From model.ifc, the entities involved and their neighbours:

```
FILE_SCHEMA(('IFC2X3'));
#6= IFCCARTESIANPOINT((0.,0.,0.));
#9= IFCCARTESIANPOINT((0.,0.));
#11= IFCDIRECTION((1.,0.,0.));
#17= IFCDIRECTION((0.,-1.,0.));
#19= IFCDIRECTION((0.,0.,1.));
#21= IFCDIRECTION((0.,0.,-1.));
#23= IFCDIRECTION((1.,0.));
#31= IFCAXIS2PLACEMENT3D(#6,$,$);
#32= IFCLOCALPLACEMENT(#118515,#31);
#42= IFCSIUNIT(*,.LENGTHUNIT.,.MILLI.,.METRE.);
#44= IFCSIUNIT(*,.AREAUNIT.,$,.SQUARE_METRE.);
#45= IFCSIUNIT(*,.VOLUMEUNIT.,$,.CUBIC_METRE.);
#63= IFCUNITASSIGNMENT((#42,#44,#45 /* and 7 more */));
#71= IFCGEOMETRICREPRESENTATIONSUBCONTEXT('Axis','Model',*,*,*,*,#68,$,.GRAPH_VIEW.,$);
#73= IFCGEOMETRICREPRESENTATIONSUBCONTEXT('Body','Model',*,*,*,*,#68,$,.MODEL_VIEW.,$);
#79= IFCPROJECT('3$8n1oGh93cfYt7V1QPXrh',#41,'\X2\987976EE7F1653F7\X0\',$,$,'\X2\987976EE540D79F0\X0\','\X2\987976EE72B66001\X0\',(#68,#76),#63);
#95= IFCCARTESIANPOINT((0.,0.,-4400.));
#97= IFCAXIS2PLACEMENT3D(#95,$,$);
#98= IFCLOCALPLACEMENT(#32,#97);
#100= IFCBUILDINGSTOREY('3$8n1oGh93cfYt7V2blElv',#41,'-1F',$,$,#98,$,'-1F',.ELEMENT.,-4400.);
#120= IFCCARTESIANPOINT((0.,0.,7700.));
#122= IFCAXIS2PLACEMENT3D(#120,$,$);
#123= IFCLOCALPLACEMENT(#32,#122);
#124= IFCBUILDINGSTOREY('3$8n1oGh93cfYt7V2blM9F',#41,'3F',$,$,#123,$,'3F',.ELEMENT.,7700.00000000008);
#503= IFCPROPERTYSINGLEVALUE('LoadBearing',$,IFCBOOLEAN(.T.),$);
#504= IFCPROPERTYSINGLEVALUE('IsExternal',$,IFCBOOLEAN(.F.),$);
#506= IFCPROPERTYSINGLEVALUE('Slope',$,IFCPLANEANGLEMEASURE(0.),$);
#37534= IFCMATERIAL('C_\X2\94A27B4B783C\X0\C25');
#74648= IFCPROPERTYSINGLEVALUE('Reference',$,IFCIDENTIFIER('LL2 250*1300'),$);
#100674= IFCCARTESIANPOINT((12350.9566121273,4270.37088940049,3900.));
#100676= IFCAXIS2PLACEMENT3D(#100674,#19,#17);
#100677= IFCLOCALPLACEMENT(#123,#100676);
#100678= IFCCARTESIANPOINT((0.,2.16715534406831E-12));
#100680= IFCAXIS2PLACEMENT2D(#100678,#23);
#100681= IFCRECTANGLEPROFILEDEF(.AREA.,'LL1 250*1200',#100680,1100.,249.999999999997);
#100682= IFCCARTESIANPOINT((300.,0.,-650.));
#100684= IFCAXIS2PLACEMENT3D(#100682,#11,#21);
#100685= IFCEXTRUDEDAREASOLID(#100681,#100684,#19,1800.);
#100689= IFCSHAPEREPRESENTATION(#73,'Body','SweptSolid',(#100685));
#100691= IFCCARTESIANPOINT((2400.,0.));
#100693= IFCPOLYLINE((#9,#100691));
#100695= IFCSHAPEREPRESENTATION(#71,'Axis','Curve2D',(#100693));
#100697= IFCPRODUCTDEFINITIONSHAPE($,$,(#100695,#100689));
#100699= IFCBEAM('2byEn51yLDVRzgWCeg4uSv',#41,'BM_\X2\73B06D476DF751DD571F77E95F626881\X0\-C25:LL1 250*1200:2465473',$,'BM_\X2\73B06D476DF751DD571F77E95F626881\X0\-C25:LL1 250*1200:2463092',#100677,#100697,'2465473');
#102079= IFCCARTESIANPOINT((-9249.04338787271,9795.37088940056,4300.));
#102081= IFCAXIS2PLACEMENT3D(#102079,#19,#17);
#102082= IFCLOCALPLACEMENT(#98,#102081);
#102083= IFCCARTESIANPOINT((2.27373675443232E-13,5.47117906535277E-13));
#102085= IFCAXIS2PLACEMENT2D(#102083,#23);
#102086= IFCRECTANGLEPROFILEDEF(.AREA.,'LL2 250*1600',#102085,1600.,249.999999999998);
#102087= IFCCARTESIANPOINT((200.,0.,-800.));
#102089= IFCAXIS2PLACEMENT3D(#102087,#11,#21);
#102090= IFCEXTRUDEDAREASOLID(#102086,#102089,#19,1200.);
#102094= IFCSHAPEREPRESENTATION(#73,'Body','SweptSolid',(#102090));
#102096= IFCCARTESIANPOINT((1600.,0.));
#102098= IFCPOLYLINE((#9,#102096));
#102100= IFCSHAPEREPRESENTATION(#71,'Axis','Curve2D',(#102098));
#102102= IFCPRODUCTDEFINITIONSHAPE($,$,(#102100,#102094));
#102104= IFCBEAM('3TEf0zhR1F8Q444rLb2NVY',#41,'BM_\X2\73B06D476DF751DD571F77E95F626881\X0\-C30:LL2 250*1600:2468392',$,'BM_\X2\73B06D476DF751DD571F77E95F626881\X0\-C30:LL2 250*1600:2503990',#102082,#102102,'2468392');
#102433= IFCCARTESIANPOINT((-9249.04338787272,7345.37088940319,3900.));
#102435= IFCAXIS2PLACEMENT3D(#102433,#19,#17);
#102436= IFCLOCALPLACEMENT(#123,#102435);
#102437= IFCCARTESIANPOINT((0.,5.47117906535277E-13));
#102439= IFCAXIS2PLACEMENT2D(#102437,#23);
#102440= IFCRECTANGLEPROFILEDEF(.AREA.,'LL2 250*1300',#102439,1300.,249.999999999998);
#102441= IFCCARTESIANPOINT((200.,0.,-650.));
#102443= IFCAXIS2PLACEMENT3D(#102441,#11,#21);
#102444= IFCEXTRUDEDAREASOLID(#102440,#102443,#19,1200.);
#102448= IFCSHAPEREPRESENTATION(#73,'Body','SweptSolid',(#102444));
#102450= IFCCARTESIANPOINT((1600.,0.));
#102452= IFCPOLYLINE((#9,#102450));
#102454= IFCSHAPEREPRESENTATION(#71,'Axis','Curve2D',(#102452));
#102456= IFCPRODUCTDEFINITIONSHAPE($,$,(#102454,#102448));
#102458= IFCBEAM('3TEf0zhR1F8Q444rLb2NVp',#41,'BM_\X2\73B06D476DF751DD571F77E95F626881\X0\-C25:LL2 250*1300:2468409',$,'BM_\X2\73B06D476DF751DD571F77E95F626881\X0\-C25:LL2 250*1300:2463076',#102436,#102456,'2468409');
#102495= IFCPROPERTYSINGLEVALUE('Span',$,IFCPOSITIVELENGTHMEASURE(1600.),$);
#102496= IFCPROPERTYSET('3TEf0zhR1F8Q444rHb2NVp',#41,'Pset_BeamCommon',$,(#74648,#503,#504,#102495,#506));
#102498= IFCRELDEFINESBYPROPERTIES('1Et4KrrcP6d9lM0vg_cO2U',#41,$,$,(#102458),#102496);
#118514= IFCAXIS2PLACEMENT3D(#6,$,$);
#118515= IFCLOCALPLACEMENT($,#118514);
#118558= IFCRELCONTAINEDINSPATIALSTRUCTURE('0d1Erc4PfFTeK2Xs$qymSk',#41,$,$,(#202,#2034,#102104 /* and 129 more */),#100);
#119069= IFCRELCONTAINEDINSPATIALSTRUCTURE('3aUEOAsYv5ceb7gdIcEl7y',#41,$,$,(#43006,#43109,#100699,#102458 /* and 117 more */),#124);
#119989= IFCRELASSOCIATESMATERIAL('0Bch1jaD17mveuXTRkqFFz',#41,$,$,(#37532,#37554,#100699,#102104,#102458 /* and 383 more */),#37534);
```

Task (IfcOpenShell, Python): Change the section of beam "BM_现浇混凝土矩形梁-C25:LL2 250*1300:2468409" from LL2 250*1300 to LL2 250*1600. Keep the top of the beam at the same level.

```python
import ifcopenshell
import ifcopenshell.api.pset
import ifcopenshell.util.element
import ifcopenshell.util.representation

model = ifcopenshell.open("model.ifc")

member = model.by_guid("3TEf0zhR1F8Q444rLb2NVp")
source = next(p for p in model.by_type("IfcRectangleProfileDef") if p.ProfileName == "LL2 250*1600")

body = ifcopenshell.util.representation.get_representation(member, "Model", "Body")
solid = body.Items[0]
old_profile = solid.SweptArea

# Copy the section's sizes but keep this member's own profile position.
profile = ifcopenshell.util.element.copy(model, source)
# Profiles are centred, so shift by half the change in depth to hold the top.
shift = (old_profile.XDim - profile.XDim) / 2
x, y = old_profile.Position.Location.Coordinates
up = (-1.0, 0.0)  # upwards, in the solid's own plane
location = model.createIfcCartesianPoint((x + up[0] * shift, y + up[1] * shift))
profile.Position = model.createIfcAxis2Placement2D(location, old_profile.Position.RefDirection)
solid.SweptArea = profile
if not model.get_total_inverses(old_profile):
    ifcopenshell.util.element.remove_deep2(model, old_profile)
member.Name = member.Name.replace("LL2 250*1300", "LL2 250*1600")
member.ObjectType = member.ObjectType.replace("LL2 250*1300", "LL2 250*1600")
pset = model.by_id(ifcopenshell.util.element.get_pset(member, "Pset_BeamCommon", should_inherit=False)["id"])
ifcopenshell.api.pset.edit_pset(model, pset=pset, properties={"Reference": "LL2 250*1600"})

print(solid.SweptArea)

model.write("model_rev.ifc")
```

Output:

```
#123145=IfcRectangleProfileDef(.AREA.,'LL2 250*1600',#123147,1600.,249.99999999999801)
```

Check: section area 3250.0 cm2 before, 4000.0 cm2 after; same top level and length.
